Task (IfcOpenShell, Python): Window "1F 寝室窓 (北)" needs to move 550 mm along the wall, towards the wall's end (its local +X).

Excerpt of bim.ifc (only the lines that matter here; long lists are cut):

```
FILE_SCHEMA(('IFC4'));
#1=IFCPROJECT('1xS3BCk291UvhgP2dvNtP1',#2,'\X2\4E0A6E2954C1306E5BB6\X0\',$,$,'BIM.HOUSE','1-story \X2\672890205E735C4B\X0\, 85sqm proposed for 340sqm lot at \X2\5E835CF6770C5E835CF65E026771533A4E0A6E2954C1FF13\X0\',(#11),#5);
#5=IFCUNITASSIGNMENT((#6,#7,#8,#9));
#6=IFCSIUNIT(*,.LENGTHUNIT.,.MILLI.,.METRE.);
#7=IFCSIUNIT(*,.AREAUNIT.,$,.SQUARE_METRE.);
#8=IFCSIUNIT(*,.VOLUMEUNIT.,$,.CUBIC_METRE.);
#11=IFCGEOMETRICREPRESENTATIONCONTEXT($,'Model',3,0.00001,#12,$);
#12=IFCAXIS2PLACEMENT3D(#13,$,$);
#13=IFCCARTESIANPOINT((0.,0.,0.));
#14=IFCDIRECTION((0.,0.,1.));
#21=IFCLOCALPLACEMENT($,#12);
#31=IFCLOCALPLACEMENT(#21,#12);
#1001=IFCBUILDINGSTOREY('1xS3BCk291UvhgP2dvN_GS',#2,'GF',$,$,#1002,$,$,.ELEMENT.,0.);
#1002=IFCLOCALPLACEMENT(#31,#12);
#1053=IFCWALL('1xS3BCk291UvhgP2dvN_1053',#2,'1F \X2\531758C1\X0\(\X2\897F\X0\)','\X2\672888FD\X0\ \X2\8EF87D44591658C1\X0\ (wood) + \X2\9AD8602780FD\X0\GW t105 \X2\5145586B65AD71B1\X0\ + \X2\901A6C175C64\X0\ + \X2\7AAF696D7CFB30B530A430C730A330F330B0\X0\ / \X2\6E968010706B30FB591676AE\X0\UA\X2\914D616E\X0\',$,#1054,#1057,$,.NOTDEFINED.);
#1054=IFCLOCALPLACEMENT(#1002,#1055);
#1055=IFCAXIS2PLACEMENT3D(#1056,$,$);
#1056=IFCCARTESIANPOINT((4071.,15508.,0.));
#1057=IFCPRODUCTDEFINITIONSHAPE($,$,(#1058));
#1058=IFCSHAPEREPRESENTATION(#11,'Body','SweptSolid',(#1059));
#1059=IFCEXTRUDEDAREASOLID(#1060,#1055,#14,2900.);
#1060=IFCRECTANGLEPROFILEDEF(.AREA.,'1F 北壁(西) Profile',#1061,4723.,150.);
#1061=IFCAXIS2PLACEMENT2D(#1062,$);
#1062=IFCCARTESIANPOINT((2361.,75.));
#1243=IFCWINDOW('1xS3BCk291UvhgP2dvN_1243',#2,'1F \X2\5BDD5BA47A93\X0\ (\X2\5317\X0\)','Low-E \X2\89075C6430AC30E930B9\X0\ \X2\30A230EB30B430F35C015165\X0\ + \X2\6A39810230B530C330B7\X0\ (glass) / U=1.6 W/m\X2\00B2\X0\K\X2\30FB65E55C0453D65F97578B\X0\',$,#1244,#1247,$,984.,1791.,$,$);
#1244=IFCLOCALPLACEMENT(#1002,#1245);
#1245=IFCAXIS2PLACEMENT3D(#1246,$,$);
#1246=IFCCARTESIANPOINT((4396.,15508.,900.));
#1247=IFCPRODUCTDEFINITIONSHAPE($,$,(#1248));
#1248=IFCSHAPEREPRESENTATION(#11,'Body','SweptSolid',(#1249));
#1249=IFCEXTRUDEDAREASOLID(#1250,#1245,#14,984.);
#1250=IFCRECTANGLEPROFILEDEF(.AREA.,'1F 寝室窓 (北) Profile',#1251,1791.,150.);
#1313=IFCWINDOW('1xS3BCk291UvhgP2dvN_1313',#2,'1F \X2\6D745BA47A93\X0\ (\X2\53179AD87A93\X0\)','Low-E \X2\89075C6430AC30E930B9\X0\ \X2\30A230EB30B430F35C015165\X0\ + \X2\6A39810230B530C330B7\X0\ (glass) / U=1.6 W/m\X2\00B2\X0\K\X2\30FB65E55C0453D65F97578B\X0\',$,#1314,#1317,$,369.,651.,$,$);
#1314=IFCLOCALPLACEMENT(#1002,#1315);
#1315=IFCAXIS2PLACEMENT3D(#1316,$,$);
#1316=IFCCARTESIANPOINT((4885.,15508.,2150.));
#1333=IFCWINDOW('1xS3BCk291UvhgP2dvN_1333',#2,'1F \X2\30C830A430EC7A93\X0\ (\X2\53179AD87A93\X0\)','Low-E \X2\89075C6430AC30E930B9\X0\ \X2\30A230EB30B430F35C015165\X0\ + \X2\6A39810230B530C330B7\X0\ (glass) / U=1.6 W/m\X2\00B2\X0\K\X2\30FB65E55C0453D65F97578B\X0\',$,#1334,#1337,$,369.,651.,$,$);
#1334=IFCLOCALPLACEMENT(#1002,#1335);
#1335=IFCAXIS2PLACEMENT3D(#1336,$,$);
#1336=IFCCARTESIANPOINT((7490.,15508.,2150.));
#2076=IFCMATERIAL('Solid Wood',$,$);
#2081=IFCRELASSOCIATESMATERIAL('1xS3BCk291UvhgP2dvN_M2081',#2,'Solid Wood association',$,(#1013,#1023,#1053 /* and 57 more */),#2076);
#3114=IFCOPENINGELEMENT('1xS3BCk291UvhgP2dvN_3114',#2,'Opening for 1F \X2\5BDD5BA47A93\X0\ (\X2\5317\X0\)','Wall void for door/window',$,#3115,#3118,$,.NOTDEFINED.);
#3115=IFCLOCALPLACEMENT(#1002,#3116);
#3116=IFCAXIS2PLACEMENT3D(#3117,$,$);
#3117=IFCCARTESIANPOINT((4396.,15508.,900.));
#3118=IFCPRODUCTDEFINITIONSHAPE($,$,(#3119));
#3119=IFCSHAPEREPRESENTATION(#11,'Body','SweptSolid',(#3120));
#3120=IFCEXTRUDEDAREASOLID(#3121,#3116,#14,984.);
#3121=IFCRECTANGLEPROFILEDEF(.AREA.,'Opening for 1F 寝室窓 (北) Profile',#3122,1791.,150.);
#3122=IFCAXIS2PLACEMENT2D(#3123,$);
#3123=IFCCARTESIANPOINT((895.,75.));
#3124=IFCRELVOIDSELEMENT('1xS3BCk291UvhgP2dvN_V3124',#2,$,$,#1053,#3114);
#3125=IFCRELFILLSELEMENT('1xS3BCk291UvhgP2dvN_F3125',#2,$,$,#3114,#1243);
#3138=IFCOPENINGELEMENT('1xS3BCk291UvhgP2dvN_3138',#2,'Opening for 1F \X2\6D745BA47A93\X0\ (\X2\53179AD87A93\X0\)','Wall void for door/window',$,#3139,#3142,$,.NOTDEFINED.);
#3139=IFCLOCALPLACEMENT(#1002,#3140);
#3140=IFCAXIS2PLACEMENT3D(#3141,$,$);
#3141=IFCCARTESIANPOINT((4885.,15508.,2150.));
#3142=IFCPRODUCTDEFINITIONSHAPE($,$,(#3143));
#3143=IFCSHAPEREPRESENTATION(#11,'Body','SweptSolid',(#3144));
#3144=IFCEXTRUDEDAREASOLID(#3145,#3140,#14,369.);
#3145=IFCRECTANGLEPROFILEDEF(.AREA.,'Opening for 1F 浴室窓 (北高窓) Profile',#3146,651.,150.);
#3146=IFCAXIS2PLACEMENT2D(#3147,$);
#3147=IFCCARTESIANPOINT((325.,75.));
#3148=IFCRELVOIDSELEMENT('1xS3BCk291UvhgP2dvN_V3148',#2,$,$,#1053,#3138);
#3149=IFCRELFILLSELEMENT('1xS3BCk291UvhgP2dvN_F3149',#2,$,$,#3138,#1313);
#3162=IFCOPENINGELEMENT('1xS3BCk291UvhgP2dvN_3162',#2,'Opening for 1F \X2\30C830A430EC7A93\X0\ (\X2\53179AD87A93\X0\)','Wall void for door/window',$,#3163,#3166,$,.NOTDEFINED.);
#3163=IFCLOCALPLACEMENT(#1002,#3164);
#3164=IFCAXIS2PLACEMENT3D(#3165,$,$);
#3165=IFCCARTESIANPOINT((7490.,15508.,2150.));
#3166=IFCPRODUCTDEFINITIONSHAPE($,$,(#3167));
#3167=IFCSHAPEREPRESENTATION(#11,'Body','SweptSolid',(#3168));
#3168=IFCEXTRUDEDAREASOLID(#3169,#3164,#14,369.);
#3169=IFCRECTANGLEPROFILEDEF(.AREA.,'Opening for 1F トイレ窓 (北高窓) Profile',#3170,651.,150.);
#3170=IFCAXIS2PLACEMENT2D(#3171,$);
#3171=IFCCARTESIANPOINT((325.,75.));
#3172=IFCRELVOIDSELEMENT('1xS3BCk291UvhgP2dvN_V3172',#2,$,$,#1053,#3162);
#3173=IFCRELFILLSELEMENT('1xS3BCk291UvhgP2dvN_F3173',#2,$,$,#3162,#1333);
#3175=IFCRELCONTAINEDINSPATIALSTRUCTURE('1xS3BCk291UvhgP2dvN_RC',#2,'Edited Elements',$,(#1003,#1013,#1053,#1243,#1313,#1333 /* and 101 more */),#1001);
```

```python
import ifcopenshell
import ifcopenshell.api.geometry
import ifcopenshell.util.placement
import ifcopenshell.util.unit

model = ifcopenshell.open("bim.ifc")
unit_scale = ifcopenshell.util.unit.calculate_unit_scale(model)

window = model.by_id(1243)
opening = window.FillsVoids[0].RelatingOpeningElement
wall = opening.VoidsElements[0].RelatingBuildingElement

wall_matrix = ifcopenshell.util.placement.get_local_placement(wall.ObjectPlacement)
shift = wall_matrix[:3, 0] * 0.55 / unit_scale
before = ifcopenshell.util.placement.get_local_placement(window.ObjectPlacement)[:3, 3].copy()

# The window is not placed relative to its opening, so move both.
for product in (opening, window):
    matrix = ifcopenshell.util.placement.get_local_placement(product.ObjectPlacement)
    matrix[:3, 3] += shift
    ifcopenshell.api.geometry.edit_object_placement(model, product=product, matrix=matrix, is_si=False)

after = ifcopenshell.util.placement.get_local_placement(window.ObjectPlacement)[:3, 3]
print("window moved by", (after - before).round(3) + 0.0)

model.write("bim-out.ifc")
```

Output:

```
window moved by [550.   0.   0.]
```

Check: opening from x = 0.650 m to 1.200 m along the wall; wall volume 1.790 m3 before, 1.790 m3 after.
